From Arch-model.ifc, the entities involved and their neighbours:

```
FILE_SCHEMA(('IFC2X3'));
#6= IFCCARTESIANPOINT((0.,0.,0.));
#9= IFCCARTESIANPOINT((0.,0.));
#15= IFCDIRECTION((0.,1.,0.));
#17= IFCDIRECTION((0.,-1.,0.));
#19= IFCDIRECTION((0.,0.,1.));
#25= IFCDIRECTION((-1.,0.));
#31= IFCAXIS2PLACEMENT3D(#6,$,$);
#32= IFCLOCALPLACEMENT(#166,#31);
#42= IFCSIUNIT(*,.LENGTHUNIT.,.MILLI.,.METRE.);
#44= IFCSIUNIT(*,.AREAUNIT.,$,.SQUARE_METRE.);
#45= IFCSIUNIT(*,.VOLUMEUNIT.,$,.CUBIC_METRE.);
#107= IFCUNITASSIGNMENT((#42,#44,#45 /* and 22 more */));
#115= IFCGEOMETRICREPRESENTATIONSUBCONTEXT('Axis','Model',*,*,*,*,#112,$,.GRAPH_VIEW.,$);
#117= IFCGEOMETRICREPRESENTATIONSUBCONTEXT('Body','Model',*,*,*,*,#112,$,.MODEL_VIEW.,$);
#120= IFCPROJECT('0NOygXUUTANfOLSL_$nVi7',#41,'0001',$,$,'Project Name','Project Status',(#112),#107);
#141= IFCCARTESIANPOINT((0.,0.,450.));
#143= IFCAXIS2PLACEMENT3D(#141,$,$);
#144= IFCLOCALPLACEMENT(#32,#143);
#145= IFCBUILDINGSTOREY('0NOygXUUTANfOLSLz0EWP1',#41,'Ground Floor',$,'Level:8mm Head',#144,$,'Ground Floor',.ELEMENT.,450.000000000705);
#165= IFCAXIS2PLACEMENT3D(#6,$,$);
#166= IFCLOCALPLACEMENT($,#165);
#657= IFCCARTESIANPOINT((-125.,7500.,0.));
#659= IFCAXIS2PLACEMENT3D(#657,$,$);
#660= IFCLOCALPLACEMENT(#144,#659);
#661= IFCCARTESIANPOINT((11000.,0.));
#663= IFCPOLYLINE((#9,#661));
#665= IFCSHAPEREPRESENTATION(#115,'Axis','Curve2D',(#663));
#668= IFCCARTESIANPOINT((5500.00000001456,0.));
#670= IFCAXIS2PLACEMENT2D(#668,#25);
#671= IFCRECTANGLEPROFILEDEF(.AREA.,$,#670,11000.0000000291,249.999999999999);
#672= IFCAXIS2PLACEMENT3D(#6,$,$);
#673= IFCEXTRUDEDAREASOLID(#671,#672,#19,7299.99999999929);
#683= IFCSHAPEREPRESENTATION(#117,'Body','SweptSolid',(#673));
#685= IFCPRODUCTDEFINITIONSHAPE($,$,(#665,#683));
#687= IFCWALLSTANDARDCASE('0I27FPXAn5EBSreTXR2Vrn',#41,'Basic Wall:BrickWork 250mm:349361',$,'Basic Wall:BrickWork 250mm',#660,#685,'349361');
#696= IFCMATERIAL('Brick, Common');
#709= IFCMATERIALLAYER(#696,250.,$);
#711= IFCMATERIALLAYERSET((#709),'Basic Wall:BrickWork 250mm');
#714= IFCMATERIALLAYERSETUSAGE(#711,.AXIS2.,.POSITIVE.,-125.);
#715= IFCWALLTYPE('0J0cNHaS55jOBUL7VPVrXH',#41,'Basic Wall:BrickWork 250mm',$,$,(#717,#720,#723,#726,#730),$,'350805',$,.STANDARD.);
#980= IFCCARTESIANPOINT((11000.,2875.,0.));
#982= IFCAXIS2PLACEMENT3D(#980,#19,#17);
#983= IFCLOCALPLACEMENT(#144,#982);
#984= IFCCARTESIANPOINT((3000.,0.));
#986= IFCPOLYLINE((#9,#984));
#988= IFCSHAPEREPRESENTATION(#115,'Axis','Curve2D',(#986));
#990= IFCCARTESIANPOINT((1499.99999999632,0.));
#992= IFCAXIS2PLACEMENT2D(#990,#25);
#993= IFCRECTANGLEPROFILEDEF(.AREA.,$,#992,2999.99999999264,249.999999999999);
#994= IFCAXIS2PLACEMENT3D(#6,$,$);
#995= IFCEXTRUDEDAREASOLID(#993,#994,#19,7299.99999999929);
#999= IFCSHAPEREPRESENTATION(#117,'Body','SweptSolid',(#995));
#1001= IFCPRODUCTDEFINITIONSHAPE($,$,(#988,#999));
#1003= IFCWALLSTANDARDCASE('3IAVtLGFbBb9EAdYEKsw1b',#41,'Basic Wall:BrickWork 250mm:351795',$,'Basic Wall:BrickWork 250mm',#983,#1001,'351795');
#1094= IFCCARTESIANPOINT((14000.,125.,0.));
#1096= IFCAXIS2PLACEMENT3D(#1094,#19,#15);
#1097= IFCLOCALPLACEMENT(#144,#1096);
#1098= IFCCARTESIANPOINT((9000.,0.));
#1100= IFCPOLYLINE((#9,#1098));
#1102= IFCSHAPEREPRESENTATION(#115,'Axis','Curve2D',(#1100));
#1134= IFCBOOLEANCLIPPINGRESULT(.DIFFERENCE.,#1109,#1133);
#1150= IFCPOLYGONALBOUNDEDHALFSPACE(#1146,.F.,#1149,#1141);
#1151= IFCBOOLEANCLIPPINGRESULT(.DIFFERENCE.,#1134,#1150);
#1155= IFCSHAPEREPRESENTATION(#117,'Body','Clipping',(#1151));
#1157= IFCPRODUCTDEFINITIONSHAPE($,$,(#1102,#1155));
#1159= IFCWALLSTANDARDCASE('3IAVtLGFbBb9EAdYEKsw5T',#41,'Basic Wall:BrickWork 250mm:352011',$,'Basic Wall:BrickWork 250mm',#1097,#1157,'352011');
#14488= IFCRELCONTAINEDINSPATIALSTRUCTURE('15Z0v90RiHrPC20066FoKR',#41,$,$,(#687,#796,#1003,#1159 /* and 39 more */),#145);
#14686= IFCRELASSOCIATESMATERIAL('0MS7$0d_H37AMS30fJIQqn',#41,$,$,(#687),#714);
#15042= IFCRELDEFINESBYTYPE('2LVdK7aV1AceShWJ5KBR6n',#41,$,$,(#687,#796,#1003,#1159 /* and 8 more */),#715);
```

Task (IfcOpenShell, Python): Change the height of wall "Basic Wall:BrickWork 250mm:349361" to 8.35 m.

```python
import ifcopenshell
import ifcopenshell.geom
import ifcopenshell.util.representation
import ifcopenshell.util.shape
import ifcopenshell.util.unit

model = ifcopenshell.open("Arch-model.ifc")
unit_scale = ifcopenshell.util.unit.calculate_unit_scale(model)
settings = ifcopenshell.geom.settings()


def volume(element):
    """Net volume in cubic metres, openings subtracted."""
    shape = ifcopenshell.geom.create_shape(settings, element)
    return ifcopenshell.util.shape.get_volume(shape.geometry)


wall = model.by_id(687)
before = volume(wall)

body = ifcopenshell.util.representation.get_representation(wall, "Model", "Body")
solid = body.Items[0]
old_height = solid.Depth
solid.Depth = 8.35 / unit_scale
after = volume(wall)

print(f"height {old_height:g} -> {solid.Depth:g}, volume {before:.3f} -> {after:.3f} m3")

model.write("Arch-model_v2.ifc")
```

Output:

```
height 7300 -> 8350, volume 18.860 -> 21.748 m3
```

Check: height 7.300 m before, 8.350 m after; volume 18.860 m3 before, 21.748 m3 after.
